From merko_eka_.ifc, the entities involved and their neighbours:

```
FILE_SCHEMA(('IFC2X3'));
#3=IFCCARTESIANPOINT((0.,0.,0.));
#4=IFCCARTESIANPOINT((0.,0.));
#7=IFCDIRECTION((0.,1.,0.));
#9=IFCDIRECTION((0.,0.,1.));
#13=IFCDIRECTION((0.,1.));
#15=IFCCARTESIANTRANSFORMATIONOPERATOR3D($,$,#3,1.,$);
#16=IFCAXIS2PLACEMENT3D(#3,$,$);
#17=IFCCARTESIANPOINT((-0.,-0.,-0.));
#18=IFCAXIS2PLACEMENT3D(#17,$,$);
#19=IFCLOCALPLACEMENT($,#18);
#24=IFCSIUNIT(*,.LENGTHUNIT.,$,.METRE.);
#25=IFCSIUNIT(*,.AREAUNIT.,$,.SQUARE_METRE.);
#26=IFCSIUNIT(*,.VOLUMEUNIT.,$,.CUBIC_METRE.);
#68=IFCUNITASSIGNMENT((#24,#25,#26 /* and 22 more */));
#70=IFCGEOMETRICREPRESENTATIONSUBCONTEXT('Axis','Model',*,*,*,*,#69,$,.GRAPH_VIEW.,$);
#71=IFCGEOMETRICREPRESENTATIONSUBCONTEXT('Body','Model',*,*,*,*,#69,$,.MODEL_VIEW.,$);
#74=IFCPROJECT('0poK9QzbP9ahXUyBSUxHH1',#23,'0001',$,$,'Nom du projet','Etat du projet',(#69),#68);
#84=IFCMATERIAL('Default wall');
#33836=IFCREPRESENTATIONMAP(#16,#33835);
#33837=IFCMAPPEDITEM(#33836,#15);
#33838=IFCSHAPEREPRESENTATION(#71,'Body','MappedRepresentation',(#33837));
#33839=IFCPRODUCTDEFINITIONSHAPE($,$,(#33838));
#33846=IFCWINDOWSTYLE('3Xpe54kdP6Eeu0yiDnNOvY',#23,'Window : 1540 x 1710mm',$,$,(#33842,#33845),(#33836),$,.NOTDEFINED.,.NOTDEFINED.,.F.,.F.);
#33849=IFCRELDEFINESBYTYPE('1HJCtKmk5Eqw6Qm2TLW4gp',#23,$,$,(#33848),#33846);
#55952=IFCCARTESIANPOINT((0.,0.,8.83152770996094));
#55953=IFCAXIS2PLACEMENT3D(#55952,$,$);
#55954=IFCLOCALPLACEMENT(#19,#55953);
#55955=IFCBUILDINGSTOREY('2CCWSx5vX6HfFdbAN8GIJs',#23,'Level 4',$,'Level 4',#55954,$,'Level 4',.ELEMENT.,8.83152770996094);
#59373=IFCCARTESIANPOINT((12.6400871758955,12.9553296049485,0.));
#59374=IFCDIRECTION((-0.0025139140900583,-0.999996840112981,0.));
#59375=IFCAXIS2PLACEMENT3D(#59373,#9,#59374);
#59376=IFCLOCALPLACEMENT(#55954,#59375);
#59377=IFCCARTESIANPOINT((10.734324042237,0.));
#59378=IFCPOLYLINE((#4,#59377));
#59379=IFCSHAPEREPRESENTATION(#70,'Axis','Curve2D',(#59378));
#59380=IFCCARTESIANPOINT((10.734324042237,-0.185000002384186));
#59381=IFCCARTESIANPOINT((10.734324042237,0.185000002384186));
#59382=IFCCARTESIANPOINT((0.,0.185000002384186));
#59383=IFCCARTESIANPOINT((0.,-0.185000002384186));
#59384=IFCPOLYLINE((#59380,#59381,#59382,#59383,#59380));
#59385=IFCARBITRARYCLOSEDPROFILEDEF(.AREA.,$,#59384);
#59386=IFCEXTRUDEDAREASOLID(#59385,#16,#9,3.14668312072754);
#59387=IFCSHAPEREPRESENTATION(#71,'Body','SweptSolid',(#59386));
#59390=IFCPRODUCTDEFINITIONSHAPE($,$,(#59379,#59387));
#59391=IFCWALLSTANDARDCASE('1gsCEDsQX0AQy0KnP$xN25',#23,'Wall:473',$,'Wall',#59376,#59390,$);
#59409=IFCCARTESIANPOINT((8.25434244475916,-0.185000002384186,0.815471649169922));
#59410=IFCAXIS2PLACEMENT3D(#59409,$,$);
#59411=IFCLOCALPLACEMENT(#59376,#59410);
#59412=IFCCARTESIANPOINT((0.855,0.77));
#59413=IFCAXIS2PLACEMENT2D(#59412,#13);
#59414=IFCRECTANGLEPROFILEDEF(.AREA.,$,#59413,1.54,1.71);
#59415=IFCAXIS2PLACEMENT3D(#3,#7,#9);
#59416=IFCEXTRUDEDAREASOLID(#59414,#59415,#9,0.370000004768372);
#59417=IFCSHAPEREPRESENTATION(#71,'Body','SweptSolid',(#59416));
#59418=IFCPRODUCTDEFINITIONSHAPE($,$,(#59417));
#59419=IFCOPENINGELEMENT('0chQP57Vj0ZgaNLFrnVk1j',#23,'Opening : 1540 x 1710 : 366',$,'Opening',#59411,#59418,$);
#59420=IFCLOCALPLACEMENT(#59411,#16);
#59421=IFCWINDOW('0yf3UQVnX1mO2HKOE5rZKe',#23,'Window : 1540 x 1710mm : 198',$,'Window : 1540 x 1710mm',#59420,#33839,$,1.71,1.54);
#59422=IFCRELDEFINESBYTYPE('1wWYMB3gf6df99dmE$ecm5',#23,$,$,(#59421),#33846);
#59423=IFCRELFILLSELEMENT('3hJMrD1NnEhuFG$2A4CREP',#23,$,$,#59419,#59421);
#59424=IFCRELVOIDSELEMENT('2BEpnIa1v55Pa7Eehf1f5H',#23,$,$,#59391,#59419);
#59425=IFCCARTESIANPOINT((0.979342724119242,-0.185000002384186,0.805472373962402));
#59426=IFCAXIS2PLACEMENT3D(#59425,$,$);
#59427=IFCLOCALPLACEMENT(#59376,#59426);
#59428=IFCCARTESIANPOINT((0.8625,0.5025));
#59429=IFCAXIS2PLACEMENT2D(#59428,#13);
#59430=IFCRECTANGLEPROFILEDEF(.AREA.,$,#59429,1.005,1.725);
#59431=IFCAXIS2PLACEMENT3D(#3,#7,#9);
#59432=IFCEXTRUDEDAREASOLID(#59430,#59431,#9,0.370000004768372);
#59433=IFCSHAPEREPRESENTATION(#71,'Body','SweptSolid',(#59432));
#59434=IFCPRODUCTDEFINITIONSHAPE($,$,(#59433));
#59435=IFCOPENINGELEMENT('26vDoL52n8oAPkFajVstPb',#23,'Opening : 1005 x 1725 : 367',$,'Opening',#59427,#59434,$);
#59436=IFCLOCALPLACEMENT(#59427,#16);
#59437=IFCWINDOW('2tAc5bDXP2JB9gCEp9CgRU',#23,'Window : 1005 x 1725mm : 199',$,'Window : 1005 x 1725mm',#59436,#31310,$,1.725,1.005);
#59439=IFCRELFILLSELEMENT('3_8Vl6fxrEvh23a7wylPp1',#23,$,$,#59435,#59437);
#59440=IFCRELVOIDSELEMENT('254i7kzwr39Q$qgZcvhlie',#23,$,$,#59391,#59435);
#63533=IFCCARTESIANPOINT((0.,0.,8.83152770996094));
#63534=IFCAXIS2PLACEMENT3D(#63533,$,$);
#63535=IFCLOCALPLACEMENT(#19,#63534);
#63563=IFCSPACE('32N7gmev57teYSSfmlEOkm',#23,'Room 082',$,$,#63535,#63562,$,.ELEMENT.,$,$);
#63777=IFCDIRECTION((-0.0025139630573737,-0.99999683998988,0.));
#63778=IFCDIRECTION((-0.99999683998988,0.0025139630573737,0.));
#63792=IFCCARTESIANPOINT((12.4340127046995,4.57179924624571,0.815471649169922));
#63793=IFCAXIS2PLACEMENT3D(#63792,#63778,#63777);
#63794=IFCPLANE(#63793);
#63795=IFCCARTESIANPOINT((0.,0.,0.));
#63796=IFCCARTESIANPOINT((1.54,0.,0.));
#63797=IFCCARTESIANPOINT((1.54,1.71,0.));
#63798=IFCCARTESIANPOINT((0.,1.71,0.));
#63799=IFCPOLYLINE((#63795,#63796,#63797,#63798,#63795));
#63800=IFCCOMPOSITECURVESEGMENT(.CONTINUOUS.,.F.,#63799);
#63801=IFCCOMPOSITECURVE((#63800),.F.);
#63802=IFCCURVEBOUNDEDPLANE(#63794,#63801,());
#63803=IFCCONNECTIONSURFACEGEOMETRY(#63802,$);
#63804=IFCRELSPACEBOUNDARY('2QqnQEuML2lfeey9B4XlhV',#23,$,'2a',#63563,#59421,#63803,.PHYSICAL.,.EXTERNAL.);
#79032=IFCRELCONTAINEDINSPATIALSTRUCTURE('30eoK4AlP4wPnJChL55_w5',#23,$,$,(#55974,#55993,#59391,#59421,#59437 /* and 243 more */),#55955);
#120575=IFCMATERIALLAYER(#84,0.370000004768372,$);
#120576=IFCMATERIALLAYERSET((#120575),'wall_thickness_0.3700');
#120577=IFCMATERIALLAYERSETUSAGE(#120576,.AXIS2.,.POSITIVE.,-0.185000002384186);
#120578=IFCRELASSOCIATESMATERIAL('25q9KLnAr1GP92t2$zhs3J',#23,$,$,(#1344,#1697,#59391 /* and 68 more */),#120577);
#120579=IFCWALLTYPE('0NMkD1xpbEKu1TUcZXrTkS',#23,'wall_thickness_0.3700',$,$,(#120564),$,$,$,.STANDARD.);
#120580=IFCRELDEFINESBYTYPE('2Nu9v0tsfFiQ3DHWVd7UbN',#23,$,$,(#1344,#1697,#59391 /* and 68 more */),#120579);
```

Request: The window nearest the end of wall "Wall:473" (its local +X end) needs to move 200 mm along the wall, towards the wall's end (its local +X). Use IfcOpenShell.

```python
import numpy as np
import ifcopenshell
import ifcopenshell.api.geometry
import ifcopenshell.util.placement

model = ifcopenshell.open("merko_eka_.ifc")

window = model.by_guid("0yf3UQVnX1mO2HKOE5rZKe")
opening = window.FillsVoids[0].RelatingOpeningElement
wall = opening.VoidsElements[0].RelatingBuildingElement

wall_matrix = ifcopenshell.util.placement.get_local_placement(wall.ObjectPlacement)
shift = wall_matrix[:3, 0] * 0.2
before = ifcopenshell.util.placement.get_local_placement(window.ObjectPlacement)[:3, 3].copy()

# The window is placed relative to its opening, so it follows when the opening moves.
matrix = ifcopenshell.util.placement.get_local_placement(opening.ObjectPlacement)
matrix[:3, 3] += shift
ifcopenshell.api.geometry.edit_object_placement(
    model, product=opening, matrix=matrix, is_si=False, should_transform_children=True
)

# Space boundary surfaces are stored in each space's coordinates; move them too.
for rel in window.ProvidesBoundaries:
    if not rel.ConnectionGeometry:
        continue
    surface = rel.ConnectionGeometry.SurfaceOnRelatingElement.BasisSurface
    space_matrix = ifcopenshell.util.placement.get_local_placement(rel.RelatingSpace.ObjectPlacement)
    point = np.array(surface.Position.Location.Coordinates) + space_matrix[:3, :3].T @ shift
    surface.Position = model.createIfcAxis2Placement3D(
        model.createIfcCartesianPoint(point.tolist()), surface.Position.Axis, surface.Position.RefDirection
    )

after = ifcopenshell.util.placement.get_local_placement(window.ObjectPlacement)[:3, 3]
print("window moved by", (after - before).round(3) + 0.0)

model.write("merko_eka__edited.ifc")
```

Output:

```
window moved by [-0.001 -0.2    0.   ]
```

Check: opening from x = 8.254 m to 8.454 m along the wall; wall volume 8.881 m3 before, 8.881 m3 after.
